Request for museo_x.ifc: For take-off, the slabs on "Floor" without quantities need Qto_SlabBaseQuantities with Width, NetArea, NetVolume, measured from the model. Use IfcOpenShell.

First a look at what the model holds.

```python
import ifcopenshell
import ifcopenshell.util.element
import ifcopenshell.util.unit

model = ifcopenshell.open("museo_x.ifc")
print(model.schema)
for unit_type in ("LENGTHUNIT", "AREAUNIT", "VOLUMEUNIT"):
    print(unit_type, ifcopenshell.util.unit.calculate_unit_scale(model, unit_type))
storey = next(s for s in model.by_type("IfcBuildingStorey") if s.Name == "Floor")
slabs = [e for e in ifcopenshell.util.element.get_decomposition(storey) if e.is_a("IfcSlab")]
for e in sorted(slabs, key=lambda e: e.id()):
    print(e.id(), e.is_a(), e.Name, list(ifcopenshell.util.element.get_psets(e, qtos_only=True)), sep=" | ")
```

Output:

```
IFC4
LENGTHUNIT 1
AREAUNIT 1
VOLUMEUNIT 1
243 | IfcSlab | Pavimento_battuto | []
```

```python
import ifcopenshell
import ifcopenshell.api.pset
import ifcopenshell.geom
import ifcopenshell.util.element
import ifcopenshell.util.shape
import ifcopenshell.util.unit

model = ifcopenshell.open("museo_x.ifc")
unit_scale = ifcopenshell.util.unit.calculate_unit_scale(model)
area_scale = ifcopenshell.util.unit.calculate_unit_scale(model, "AREAUNIT")
volume_scale = ifcopenshell.util.unit.calculate_unit_scale(model, "VOLUMEUNIT")
settings = ifcopenshell.geom.settings()

storey = next(s for s in model.by_type("IfcBuildingStorey") if s.Name == "Floor")
slabs = [e for e in ifcopenshell.util.element.get_decomposition(storey) if e.is_a("IfcSlab")]

for e in sorted(slabs, key=lambda e: e.id()):
    if ifcopenshell.util.element.get_psets(e, qtos_only=True, should_inherit=False):
        continue
    # Geometry comes back in metres, in the element's own axes.
    shape = ifcopenshell.geom.create_shape(settings, e)
    values = {
        "Width": ifcopenshell.util.shape.get_z(shape.geometry) / unit_scale,
        "NetArea": ifcopenshell.util.shape.get_footprint_area(shape.geometry) / area_scale,
        "NetVolume": ifcopenshell.util.shape.get_volume(shape.geometry) / volume_scale,
    }
    qto = ifcopenshell.api.pset.add_qto(model, product=e, name="Qto_SlabBaseQuantities")
    ifcopenshell.api.pset.edit_qto(model, qto=qto, properties=values)
    print(e.id(), {k: round(v, 3) for k, v in values.items()})

model.write("museo_x_rev.ifc")
```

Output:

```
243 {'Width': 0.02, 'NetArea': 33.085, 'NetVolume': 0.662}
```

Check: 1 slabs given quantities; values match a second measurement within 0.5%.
